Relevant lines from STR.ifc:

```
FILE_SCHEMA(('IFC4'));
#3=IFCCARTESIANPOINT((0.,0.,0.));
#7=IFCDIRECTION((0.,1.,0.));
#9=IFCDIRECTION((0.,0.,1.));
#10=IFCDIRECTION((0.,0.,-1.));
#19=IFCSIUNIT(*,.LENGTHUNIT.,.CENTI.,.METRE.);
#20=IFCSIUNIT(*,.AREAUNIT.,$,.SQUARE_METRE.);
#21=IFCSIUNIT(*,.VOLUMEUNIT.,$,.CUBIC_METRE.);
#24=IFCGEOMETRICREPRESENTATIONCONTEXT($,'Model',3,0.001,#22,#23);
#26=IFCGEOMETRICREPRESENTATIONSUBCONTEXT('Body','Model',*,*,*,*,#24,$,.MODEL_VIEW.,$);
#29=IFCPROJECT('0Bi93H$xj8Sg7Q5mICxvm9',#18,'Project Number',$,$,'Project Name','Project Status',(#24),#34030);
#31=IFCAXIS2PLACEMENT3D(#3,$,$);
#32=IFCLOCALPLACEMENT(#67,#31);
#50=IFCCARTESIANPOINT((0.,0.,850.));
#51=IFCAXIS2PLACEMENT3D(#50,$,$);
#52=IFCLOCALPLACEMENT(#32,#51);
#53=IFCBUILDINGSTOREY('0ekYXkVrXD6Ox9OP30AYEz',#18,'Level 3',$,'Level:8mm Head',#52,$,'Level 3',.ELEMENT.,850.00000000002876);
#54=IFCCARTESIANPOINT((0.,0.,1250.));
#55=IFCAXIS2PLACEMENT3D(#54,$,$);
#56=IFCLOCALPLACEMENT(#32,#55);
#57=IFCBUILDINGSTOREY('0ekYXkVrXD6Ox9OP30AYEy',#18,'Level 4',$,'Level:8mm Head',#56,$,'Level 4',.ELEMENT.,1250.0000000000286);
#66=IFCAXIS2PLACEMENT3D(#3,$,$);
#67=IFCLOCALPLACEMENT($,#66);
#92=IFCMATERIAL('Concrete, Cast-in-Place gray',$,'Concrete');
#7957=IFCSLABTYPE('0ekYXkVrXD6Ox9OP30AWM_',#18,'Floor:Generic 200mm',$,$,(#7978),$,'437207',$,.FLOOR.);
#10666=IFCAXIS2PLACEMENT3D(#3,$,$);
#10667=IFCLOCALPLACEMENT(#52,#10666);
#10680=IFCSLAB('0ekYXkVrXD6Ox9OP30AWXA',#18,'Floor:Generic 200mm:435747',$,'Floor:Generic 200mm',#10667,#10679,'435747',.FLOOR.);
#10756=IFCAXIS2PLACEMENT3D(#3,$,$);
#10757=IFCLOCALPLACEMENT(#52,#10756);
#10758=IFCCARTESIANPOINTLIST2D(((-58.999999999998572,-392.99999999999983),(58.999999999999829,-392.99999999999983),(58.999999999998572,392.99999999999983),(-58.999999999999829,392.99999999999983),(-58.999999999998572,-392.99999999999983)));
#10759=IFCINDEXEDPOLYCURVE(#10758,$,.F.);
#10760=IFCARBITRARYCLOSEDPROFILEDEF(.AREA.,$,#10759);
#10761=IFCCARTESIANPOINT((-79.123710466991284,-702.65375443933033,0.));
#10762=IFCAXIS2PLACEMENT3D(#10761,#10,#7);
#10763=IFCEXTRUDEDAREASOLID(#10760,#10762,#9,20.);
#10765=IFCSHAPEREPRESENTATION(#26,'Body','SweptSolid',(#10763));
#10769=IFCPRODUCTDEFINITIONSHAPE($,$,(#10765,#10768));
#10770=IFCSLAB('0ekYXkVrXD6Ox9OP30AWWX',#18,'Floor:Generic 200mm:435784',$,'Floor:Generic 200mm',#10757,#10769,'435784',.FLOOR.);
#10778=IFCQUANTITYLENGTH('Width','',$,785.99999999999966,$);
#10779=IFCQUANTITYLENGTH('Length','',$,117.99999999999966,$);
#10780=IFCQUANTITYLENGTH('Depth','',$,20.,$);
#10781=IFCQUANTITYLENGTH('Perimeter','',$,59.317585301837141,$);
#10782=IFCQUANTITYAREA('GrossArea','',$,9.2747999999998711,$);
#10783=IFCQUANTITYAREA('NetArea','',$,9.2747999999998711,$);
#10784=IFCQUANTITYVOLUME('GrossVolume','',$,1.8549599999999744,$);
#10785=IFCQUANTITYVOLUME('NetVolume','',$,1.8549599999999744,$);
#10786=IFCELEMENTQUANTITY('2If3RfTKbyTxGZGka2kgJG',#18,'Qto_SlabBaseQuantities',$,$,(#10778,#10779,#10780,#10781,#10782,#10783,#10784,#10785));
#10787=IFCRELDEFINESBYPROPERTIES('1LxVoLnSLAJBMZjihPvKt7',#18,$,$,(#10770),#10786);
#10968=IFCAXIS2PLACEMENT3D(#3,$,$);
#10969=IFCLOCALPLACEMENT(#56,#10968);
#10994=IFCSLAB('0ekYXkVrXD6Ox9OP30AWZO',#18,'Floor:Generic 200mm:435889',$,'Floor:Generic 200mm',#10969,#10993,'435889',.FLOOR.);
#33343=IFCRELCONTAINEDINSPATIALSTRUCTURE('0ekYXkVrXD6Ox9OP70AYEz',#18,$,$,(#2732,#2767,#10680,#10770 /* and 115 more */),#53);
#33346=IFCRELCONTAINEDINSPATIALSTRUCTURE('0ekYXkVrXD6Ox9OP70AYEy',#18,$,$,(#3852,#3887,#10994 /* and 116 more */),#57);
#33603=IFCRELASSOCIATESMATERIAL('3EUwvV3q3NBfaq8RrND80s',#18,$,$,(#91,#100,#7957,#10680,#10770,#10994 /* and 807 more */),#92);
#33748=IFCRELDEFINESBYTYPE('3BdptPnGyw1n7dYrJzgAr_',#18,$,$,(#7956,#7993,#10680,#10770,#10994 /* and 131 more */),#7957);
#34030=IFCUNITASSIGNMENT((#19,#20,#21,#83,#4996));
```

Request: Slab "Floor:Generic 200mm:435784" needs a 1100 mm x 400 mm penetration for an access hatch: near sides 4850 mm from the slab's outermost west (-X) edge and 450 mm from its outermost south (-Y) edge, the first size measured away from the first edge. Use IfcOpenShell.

```python
import numpy as np
import ifcopenshell
import ifcopenshell.api.feature
import ifcopenshell.api.geometry
import ifcopenshell.api.pset
import ifcopenshell.api.root
import ifcopenshell.geom
import ifcopenshell.util.element
import ifcopenshell.util.placement
import ifcopenshell.util.representation
import ifcopenshell.util.shape
import ifcopenshell.util.unit

model = ifcopenshell.open("STR.ifc")
unit_scale = ifcopenshell.util.unit.calculate_unit_scale(model)
area_scale = ifcopenshell.util.unit.calculate_unit_scale(model, "AREAUNIT")
volume_scale = ifcopenshell.util.unit.calculate_unit_scale(model, "VOLUMEUNIT")
settings = ifcopenshell.geom.settings()


def volume(element):
    """Net volume in cubic metres, openings subtracted."""
    shape = ifcopenshell.geom.create_shape(settings, element)
    return ifcopenshell.util.shape.get_volume(shape.geometry)


slab = model.by_guid("0ekYXkVrXD6Ox9OP30AWWX")
before = volume(slab)

# Extent in the slab's own axes, in metres. The edges named are its -X and -Y sides.
slab_shape = ifcopenshell.geom.create_shape(settings, slab)
vertices = ifcopenshell.util.shape.get_vertices(slab_shape.geometry)
x_min, y_min, bottom = vertices.min(axis=0)
top = vertices[:, 2].max()

opening = ifcopenshell.api.root.create_entity(model, ifc_class="IfcOpeningElement", name="Access hatch opening", predefined_type="OPENING")
context = ifcopenshell.util.representation.get_context(model, "Model", "Body", "MODEL_VIEW")
width, depth = 1.1, 0.4
outline = [(0.0, 0.0), (width, 0.0), (width, depth), (0.0, depth), (0.0, 0.0)]
# Overshoot both faces by 50 mm so the cut is clean.
shape = ifcopenshell.api.geometry.add_slab_representation(
    model, context=context, depth=top - bottom + 0.1, polyline=outline
)
ifcopenshell.api.geometry.assign_representation(model, product=opening, representation=shape)

matrix = ifcopenshell.util.placement.get_local_placement(slab.ObjectPlacement)
matrix[:, 3] = matrix @ np.append(np.array([x_min + 4.85, y_min + 0.45, bottom - 0.05]) / unit_scale, 1.0)
ifcopenshell.api.geometry.edit_object_placement(model, product=opening, matrix=matrix, is_si=False)
ifcopenshell.api.feature.add_feature(model, feature=opening, element=slab)

after = volume(slab)

# Update the slab's stored quantities.
qto = model.by_id(ifcopenshell.util.element.get_pset(slab, "Qto_SlabBaseQuantities", should_inherit=False)["id"])
ifcopenshell.api.pset.edit_qto(model, qto=qto, properties={
    "NetArea": after / (top - bottom) / area_scale,
    "NetVolume": after / volume_scale,
})

print(f"slab volume {before:.3f} -> {after:.3f} m3")

model.write("STR_v2.ifc")
```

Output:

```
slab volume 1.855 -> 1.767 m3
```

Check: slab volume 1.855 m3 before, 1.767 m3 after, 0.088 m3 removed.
